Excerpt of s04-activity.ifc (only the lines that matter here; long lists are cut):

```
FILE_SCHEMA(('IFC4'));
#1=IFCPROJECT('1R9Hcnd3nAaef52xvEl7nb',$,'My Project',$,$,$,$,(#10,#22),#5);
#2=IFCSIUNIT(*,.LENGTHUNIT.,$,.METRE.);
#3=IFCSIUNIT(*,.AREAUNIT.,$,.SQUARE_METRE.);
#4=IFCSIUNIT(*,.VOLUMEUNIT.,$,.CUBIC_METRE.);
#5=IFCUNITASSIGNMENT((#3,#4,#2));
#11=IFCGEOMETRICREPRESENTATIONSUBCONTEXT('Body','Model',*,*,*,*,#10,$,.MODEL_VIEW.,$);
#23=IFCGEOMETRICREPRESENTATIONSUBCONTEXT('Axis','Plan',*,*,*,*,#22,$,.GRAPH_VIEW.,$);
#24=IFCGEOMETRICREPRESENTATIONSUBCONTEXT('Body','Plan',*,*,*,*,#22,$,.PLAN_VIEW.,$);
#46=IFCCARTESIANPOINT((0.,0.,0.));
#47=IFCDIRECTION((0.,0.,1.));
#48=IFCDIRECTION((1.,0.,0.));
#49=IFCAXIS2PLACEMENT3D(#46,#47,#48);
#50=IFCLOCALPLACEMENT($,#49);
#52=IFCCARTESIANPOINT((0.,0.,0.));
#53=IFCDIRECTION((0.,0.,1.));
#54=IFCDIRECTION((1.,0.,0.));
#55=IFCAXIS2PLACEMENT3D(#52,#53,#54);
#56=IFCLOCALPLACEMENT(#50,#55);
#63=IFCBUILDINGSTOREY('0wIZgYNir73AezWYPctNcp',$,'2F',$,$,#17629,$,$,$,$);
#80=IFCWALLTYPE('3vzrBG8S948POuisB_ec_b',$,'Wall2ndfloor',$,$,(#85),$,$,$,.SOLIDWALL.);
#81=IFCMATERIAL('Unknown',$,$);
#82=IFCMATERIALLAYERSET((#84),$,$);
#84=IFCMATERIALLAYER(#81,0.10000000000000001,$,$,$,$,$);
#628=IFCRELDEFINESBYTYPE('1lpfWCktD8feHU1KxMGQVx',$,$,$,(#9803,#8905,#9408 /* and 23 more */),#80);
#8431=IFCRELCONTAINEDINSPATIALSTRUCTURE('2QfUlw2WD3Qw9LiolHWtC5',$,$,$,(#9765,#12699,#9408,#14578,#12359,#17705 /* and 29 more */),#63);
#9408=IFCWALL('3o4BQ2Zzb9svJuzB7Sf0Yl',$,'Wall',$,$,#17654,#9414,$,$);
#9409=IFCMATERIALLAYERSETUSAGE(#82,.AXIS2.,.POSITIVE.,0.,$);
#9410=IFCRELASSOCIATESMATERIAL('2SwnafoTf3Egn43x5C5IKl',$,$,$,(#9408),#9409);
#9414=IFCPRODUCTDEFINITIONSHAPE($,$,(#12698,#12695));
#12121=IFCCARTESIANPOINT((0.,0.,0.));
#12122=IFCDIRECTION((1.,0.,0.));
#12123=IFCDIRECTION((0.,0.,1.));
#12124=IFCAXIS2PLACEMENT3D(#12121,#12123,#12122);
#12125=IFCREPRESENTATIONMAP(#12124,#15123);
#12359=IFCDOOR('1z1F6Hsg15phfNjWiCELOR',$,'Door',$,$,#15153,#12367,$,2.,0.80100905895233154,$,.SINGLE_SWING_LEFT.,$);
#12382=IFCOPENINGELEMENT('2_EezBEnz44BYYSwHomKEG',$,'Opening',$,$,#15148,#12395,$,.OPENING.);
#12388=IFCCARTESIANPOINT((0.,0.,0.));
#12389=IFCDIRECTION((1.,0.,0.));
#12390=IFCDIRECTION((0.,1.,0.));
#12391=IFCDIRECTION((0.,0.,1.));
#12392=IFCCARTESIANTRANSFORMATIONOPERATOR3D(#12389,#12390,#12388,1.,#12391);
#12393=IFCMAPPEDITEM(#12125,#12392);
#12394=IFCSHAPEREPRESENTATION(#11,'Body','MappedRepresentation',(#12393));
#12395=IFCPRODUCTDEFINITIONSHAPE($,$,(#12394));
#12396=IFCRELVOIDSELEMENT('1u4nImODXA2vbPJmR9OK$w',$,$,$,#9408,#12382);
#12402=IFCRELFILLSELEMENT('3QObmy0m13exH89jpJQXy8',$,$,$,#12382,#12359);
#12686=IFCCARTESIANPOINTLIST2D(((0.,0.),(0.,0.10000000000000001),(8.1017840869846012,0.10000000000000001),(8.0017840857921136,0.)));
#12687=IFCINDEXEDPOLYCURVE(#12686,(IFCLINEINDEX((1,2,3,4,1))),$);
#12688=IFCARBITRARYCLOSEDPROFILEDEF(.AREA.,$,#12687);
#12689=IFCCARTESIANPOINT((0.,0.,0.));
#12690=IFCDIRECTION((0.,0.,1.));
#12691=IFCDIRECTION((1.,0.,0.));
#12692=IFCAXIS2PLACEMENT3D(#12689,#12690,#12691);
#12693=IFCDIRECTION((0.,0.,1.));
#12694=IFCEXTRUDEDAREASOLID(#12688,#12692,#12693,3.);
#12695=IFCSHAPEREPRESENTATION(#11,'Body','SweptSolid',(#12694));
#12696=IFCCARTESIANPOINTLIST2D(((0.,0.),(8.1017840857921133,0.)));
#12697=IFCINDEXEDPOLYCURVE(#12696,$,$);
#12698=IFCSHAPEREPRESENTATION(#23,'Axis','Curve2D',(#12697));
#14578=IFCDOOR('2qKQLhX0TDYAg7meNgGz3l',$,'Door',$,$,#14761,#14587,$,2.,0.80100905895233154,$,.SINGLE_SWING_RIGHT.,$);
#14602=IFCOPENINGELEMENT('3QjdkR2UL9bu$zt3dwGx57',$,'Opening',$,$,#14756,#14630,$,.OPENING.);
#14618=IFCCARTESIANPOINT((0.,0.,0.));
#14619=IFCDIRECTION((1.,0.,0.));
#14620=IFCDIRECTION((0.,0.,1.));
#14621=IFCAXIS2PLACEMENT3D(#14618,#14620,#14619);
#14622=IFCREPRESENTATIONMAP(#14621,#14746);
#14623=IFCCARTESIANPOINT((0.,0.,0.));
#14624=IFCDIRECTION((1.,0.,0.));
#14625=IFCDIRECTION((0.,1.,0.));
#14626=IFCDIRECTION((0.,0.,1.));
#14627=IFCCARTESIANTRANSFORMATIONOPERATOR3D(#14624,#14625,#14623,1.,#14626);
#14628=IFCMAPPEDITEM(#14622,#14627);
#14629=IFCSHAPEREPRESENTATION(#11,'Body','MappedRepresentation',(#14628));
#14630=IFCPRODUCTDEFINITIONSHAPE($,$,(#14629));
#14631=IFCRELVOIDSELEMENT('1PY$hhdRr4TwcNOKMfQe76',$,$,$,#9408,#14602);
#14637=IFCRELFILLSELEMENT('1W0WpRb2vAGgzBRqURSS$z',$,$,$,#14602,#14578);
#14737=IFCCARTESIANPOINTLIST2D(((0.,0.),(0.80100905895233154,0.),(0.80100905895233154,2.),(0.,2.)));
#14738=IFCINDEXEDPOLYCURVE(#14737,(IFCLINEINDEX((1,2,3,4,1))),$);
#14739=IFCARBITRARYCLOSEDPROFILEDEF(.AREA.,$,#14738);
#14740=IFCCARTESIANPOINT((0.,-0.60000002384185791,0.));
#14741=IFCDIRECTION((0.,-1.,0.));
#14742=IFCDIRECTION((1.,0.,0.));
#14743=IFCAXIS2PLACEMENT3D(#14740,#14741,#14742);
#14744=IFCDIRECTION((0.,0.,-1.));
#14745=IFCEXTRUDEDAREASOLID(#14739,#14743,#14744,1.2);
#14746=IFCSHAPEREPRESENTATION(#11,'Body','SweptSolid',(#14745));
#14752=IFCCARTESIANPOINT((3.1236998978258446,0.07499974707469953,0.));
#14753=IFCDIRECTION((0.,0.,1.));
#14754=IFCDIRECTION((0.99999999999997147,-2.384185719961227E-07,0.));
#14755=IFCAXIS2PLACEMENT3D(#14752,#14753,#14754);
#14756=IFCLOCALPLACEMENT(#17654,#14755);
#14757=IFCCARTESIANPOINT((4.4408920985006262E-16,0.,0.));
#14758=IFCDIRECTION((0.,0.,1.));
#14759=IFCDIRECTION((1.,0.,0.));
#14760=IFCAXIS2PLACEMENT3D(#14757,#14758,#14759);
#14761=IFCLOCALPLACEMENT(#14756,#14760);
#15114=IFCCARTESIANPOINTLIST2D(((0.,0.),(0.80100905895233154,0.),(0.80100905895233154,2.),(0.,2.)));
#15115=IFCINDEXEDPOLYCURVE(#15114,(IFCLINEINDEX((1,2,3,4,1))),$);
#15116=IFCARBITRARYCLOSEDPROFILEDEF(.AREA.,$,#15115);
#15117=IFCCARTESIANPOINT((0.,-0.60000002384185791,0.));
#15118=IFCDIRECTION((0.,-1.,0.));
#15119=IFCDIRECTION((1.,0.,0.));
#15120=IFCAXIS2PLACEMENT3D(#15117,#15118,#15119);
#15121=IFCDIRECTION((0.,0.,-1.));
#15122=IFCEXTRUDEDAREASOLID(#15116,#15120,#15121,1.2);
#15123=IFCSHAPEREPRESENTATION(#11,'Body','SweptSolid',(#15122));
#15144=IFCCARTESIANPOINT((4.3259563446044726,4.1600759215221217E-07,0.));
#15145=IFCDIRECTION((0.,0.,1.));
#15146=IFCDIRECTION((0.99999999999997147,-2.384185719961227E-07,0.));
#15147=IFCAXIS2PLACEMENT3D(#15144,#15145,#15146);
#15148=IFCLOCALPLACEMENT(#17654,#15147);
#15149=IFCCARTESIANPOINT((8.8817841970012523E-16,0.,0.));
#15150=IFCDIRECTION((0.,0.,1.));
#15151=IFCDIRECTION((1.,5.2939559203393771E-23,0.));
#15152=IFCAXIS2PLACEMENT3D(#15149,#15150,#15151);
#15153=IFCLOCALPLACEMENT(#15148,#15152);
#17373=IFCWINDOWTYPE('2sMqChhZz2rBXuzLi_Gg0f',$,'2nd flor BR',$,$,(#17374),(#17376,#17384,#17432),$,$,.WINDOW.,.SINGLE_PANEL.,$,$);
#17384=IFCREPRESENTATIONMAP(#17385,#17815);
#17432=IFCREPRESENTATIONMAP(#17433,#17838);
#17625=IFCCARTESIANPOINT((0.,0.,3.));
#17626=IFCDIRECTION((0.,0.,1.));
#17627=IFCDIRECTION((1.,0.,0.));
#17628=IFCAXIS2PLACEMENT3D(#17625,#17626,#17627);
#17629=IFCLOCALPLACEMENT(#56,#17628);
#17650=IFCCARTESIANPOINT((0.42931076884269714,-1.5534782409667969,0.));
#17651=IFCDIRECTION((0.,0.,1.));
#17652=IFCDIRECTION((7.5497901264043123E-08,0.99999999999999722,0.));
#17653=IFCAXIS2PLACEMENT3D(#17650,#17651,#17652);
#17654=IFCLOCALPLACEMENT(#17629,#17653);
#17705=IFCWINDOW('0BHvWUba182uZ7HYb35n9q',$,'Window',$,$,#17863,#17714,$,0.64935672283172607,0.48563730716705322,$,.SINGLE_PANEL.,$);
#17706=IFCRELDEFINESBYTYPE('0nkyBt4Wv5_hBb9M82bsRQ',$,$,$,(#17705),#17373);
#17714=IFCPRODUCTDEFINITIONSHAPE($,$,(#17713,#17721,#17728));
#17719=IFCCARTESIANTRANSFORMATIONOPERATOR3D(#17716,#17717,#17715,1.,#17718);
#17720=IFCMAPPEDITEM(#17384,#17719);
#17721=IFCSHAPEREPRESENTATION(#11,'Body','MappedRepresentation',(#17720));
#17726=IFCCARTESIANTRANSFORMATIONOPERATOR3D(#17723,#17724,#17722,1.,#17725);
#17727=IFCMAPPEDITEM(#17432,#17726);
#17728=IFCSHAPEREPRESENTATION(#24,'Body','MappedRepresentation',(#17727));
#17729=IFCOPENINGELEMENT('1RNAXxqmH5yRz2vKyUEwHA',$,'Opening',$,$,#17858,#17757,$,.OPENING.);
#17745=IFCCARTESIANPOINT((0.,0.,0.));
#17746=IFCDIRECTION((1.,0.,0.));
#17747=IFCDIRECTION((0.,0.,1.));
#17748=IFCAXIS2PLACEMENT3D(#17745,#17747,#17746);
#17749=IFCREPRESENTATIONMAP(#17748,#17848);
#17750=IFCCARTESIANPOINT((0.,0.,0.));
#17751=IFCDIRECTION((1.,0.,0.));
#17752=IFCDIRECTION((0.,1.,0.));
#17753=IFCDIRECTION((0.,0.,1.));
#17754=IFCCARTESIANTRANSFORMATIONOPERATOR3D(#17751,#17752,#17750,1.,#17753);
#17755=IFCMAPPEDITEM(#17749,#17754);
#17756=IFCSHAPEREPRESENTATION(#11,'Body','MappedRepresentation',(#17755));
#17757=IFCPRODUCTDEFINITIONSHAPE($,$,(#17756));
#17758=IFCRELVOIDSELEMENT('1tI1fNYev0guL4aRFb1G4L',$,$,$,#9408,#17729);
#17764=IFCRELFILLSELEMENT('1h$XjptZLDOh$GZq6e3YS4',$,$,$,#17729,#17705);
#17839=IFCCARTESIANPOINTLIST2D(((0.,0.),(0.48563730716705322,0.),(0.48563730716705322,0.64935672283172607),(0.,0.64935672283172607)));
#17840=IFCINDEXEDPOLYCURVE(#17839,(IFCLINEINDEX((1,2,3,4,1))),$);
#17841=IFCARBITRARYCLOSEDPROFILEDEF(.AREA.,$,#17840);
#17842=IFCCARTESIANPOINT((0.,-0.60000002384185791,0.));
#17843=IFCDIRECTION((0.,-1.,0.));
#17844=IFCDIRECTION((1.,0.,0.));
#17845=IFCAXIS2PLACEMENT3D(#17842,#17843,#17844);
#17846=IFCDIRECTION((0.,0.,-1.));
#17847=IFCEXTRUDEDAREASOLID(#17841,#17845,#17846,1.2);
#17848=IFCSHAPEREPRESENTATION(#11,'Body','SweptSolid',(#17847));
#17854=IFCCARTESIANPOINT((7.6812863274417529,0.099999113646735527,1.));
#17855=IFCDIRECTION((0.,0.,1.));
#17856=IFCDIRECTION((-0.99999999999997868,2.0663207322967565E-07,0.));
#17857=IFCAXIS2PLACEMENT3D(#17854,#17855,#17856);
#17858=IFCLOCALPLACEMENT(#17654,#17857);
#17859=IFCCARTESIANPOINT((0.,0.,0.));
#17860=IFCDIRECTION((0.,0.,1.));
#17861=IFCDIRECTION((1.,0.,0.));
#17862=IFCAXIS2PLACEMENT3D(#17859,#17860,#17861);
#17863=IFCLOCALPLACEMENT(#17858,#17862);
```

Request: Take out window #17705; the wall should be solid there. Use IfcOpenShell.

```python
import ifcopenshell
import ifcopenshell.api.feature
import ifcopenshell.api.root
import ifcopenshell.geom
import ifcopenshell.util.shape

model = ifcopenshell.open("s04-activity.ifc")
settings = ifcopenshell.geom.settings()


def volume(element):
    """Net volume in cubic metres, openings subtracted."""
    shape = ifcopenshell.geom.create_shape(settings, element)
    return ifcopenshell.util.shape.get_volume(shape.geometry)


window = model.by_guid("0BHvWUba182uZ7HYb35n9q")
opening = window.FillsVoids[0].RelatingOpeningElement
wall = opening.VoidsElements[0].RelatingBuildingElement
before = volume(wall)

ifcopenshell.api.root.remove_product(model, product=window)
ifcopenshell.api.feature.remove_feature(model, feature=opening)

after = volume(wall)

print(f"wall volume {before:.3f} -> {after:.3f} m3")

model.write("s04-activity_v2.ifc")
```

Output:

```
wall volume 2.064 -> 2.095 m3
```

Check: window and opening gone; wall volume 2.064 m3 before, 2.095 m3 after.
